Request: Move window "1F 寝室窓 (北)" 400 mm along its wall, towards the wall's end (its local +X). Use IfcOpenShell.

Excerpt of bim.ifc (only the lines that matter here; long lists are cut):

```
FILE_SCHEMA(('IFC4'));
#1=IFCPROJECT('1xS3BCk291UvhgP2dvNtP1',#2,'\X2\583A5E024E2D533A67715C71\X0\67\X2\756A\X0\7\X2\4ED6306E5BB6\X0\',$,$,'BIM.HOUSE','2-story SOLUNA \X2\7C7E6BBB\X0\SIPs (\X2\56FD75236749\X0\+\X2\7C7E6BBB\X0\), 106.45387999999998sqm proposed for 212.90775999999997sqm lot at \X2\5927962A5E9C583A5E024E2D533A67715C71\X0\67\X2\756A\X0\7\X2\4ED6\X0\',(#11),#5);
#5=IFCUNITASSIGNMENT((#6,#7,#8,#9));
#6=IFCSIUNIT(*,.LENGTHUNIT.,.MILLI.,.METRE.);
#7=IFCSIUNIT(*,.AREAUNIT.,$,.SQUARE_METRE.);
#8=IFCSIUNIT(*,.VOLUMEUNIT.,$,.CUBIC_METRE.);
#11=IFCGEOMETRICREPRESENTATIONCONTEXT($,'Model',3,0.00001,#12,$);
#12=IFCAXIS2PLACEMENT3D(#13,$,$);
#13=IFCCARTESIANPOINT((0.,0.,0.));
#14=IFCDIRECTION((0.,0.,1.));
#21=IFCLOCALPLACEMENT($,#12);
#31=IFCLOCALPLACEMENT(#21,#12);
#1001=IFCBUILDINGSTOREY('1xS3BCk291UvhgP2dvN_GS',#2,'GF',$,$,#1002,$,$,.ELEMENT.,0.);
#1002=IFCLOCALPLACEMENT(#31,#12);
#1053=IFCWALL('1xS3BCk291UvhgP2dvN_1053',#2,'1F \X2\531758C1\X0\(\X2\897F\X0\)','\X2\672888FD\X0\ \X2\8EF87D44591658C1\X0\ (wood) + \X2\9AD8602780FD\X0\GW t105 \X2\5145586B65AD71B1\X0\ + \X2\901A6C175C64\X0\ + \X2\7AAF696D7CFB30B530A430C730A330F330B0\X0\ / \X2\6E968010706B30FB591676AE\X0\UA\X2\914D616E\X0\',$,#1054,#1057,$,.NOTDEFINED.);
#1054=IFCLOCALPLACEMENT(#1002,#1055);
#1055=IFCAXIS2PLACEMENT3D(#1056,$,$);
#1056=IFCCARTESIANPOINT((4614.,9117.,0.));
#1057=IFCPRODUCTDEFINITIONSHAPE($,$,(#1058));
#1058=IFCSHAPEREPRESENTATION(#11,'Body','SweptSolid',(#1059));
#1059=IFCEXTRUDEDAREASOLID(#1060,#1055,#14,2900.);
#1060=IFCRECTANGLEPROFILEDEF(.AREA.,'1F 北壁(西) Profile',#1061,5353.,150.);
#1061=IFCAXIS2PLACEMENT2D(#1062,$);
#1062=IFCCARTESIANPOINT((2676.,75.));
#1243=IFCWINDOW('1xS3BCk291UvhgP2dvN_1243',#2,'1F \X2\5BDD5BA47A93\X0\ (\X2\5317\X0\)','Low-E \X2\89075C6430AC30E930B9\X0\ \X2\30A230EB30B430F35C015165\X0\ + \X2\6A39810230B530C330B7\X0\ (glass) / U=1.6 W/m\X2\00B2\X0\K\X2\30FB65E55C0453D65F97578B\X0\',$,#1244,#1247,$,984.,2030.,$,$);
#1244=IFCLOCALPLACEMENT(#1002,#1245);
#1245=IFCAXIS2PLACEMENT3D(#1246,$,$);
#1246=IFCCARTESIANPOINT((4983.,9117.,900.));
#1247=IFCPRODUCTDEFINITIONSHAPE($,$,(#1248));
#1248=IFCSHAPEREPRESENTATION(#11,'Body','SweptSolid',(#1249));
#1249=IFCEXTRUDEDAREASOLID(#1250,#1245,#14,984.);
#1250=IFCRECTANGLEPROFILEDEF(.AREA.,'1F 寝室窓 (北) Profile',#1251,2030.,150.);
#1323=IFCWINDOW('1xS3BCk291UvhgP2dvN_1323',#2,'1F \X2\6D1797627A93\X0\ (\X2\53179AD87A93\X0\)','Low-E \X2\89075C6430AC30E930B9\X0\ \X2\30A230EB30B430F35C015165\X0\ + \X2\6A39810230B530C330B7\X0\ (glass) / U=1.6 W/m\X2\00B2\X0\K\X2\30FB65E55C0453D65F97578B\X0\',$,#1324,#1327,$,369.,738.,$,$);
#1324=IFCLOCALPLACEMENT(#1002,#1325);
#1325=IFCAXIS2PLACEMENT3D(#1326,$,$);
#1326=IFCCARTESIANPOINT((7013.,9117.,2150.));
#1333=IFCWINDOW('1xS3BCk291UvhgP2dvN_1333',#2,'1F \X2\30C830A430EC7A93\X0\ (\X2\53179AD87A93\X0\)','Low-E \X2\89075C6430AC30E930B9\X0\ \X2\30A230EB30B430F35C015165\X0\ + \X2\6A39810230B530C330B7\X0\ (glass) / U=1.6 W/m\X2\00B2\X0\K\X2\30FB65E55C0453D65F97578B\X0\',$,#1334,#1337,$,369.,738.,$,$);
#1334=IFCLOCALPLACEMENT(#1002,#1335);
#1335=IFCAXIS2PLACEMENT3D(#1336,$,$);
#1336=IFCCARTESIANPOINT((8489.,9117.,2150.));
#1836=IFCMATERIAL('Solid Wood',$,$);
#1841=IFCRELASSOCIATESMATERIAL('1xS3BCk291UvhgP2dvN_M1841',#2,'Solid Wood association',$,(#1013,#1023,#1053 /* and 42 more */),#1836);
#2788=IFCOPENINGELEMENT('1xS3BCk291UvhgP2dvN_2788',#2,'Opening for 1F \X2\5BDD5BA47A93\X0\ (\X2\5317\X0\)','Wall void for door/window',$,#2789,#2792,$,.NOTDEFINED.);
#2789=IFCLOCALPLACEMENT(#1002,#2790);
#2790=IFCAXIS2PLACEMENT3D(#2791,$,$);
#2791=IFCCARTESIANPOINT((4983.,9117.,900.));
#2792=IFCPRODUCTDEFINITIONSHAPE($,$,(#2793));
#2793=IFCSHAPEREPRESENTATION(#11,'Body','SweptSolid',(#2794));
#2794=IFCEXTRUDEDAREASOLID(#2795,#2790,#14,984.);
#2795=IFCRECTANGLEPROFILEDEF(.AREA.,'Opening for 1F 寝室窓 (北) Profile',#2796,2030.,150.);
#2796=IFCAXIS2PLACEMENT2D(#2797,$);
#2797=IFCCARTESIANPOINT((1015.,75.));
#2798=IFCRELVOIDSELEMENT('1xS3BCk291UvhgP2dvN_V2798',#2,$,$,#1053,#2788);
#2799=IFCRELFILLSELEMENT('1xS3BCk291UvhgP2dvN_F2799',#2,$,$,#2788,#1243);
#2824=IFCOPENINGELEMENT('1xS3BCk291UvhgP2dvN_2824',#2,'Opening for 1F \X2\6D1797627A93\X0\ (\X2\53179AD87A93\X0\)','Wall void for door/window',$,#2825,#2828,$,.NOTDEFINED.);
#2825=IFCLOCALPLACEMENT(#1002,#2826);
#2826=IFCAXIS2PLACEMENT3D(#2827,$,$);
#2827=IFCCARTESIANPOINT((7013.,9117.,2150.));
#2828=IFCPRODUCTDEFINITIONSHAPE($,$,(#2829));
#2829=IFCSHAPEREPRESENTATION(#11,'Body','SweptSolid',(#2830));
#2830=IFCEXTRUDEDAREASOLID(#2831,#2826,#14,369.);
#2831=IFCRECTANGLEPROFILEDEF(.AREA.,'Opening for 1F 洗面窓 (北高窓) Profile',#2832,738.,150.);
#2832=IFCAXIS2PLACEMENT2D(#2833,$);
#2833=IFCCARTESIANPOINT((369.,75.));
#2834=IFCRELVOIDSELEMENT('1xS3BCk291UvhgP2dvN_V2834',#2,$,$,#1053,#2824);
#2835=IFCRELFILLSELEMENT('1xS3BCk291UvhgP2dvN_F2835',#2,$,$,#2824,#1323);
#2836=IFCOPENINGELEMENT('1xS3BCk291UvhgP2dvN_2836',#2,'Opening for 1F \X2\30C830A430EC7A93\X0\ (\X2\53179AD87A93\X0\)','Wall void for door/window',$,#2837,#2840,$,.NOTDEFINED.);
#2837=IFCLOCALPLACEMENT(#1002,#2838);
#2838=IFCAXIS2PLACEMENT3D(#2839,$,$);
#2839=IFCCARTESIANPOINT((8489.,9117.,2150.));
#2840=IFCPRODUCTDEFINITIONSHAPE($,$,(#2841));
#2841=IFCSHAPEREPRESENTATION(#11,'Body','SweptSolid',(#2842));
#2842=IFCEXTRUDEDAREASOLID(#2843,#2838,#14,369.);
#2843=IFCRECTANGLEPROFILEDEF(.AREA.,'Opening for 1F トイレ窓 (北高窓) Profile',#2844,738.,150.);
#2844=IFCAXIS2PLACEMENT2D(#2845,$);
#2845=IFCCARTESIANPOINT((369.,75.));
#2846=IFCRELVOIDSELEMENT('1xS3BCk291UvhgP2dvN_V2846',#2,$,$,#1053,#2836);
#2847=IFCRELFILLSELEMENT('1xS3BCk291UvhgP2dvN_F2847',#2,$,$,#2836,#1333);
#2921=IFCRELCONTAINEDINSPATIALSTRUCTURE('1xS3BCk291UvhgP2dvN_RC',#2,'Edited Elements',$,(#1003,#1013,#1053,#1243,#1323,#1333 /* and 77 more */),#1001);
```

```python
import ifcopenshell
import ifcopenshell.api.geometry
import ifcopenshell.util.placement

model = ifcopenshell.open("bim.ifc")

window = model.by_guid("1xS3BCk291UvhgP2dvN_1243")
opening = window.FillsVoids[0].RelatingOpeningElement
wall = opening.VoidsElements[0].RelatingBuildingElement

wall_matrix = ifcopenshell.util.placement.get_local_placement(wall.ObjectPlacement)
shift = wall_matrix[:3, 0] * 400.0
before = ifcopenshell.util.placement.get_local_placement(window.ObjectPlacement)[:3, 3].copy()

# The window is not placed relative to its opening, so move both.
for product in (opening, window):
    matrix = ifcopenshell.util.placement.get_local_placement(product.ObjectPlacement)
    matrix[:3, 3] += shift
    ifcopenshell.api.geometry.edit_object_placement(model, product=product, matrix=matrix, is_si=False)

after = ifcopenshell.util.placement.get_local_placement(window.ObjectPlacement)[:3, 3]
print("window moved by", (after - before).round(3) + 0.0)

model.write("bim-out.ifc")
```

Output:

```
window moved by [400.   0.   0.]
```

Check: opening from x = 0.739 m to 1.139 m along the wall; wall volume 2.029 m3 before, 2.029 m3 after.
